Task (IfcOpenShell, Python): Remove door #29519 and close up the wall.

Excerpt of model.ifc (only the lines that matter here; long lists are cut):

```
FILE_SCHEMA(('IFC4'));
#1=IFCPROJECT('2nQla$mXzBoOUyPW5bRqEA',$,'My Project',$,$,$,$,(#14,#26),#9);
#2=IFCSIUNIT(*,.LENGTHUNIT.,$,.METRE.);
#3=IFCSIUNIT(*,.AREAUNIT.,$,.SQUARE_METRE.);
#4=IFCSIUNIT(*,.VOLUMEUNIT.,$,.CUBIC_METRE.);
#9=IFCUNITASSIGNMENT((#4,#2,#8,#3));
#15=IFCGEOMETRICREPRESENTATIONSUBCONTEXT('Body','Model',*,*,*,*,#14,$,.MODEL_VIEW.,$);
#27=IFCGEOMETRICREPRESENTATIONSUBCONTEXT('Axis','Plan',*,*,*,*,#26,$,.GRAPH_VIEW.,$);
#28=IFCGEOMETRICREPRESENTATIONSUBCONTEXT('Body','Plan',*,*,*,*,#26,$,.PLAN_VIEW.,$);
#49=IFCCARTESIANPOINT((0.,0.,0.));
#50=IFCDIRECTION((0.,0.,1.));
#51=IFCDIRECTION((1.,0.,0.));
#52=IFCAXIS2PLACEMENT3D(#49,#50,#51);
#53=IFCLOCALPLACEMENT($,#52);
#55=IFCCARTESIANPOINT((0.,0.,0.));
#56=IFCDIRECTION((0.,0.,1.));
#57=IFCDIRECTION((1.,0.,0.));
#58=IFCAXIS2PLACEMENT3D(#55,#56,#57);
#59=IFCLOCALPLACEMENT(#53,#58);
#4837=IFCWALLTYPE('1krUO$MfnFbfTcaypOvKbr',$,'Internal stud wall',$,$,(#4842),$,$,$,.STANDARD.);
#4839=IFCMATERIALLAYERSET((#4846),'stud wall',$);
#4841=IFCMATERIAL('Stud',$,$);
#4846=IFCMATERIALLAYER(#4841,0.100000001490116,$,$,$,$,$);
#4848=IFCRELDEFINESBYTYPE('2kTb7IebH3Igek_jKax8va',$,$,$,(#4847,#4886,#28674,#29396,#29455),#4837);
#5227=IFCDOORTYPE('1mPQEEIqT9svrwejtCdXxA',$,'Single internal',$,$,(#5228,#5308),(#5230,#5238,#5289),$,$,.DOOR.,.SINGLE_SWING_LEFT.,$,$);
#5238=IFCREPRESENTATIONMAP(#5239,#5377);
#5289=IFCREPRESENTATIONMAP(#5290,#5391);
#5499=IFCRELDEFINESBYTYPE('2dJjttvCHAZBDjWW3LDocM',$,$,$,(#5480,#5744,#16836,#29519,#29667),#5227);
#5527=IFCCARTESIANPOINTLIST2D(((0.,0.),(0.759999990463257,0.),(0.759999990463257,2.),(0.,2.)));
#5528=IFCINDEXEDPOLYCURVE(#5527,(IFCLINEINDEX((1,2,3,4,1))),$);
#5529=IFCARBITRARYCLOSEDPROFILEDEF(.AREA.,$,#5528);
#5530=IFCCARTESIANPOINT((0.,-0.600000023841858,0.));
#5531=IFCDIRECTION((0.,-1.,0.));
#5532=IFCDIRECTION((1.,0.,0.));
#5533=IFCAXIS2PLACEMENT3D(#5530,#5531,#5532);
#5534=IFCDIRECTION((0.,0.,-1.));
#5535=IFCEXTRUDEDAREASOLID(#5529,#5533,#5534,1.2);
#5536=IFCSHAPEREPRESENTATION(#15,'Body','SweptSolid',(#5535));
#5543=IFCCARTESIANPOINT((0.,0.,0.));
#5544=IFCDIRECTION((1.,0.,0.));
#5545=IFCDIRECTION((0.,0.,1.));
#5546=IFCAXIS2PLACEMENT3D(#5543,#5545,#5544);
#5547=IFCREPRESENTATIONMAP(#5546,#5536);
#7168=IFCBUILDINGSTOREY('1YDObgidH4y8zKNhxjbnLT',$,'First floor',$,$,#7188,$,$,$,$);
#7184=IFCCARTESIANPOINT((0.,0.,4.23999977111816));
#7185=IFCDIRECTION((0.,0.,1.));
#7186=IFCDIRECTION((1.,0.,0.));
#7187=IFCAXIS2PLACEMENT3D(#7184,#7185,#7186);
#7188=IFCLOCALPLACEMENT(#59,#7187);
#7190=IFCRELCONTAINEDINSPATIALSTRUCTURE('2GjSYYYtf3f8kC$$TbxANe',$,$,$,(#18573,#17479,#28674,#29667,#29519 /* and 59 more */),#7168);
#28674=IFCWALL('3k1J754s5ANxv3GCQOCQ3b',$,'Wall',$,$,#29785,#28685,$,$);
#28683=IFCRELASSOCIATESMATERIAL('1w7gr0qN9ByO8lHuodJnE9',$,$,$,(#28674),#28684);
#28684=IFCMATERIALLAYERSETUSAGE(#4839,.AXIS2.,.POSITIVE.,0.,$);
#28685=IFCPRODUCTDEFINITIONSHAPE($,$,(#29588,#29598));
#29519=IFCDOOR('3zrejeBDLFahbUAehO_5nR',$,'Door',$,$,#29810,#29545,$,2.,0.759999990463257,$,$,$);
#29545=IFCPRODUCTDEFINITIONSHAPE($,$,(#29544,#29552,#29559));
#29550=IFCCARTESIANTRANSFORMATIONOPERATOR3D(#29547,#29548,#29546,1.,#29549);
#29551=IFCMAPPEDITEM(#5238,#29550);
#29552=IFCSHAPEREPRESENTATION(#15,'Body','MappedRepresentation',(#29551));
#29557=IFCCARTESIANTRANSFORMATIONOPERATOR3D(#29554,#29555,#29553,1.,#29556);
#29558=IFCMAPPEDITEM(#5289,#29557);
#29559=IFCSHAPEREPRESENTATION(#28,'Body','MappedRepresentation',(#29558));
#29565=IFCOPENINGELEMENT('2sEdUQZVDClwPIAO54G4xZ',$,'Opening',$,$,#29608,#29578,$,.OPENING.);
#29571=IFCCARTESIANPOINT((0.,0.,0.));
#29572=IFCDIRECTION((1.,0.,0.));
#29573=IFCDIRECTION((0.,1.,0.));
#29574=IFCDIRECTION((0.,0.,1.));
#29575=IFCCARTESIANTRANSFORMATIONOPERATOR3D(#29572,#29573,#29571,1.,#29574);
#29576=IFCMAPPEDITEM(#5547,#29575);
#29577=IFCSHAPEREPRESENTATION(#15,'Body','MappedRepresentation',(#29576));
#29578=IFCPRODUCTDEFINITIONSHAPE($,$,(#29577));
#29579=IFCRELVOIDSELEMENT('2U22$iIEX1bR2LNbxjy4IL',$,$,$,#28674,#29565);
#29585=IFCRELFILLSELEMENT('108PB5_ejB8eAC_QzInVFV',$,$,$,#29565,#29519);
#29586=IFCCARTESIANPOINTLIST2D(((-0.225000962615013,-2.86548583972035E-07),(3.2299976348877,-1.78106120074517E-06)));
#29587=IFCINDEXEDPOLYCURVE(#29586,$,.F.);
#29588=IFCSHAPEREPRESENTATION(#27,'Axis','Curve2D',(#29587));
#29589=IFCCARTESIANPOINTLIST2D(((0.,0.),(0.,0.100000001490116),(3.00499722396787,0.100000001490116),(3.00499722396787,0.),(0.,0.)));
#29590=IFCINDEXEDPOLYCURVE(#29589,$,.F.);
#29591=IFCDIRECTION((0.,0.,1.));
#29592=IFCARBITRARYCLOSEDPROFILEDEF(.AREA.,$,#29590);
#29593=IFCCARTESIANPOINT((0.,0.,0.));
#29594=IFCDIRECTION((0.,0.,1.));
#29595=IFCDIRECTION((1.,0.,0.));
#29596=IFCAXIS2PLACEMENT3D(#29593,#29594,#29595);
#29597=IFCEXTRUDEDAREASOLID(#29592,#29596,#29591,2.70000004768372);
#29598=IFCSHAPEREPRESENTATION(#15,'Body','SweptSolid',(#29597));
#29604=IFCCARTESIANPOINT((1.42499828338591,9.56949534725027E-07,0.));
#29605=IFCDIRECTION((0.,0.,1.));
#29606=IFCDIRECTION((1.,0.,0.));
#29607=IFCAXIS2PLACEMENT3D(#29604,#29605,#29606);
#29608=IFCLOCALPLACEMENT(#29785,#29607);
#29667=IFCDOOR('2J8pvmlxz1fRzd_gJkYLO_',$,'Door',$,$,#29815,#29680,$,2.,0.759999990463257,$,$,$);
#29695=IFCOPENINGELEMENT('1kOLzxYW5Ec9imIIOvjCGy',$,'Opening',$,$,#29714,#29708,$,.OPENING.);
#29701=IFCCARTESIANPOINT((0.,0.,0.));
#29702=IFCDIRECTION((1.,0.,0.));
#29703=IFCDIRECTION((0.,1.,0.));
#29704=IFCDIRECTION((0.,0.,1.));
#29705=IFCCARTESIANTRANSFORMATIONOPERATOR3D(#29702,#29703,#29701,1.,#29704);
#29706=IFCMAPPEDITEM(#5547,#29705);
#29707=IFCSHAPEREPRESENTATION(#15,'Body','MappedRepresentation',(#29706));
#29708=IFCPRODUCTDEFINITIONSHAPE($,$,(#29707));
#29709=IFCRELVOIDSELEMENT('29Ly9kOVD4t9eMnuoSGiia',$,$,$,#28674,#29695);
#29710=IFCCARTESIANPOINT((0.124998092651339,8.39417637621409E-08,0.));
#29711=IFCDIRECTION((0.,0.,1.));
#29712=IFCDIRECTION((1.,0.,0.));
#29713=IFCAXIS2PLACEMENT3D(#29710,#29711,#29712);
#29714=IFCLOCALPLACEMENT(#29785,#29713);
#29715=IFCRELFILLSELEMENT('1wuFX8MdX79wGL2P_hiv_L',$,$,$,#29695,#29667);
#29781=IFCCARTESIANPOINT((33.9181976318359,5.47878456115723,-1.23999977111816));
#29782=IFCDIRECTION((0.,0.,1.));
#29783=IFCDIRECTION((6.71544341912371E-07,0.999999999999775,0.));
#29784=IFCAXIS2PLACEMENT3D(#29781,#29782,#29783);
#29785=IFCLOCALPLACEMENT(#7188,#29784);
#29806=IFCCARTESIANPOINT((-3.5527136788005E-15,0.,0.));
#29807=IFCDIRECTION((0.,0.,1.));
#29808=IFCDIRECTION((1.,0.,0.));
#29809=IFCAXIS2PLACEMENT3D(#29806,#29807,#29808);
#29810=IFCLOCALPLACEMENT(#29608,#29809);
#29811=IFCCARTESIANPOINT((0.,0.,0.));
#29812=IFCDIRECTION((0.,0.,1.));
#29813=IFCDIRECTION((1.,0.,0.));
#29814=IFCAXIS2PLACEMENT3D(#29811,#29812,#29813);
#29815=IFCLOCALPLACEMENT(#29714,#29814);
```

```python
import ifcopenshell
import ifcopenshell.api.feature
import ifcopenshell.api.root
import ifcopenshell.geom
import ifcopenshell.util.shape

model = ifcopenshell.open("model.ifc")
settings = ifcopenshell.geom.settings()


def volume(element):
    """Net volume in cubic metres, openings subtracted."""
    shape = ifcopenshell.geom.create_shape(settings, element)
    return ifcopenshell.util.shape.get_volume(shape.geometry)


door = model.by_guid("3zrejeBDLFahbUAehO_5nR")
opening = door.FillsVoids[0].RelatingOpeningElement
wall = opening.VoidsElements[0].RelatingBuildingElement
before = volume(wall)

ifcopenshell.api.root.remove_product(model, product=door)
ifcopenshell.api.feature.remove_feature(model, feature=opening)

after = volume(wall)

print(f"wall volume {before:.3f} -> {after:.3f} m3")

model.write("model_edited.ifc")
```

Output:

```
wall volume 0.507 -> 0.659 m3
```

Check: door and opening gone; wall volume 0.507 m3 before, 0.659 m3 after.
